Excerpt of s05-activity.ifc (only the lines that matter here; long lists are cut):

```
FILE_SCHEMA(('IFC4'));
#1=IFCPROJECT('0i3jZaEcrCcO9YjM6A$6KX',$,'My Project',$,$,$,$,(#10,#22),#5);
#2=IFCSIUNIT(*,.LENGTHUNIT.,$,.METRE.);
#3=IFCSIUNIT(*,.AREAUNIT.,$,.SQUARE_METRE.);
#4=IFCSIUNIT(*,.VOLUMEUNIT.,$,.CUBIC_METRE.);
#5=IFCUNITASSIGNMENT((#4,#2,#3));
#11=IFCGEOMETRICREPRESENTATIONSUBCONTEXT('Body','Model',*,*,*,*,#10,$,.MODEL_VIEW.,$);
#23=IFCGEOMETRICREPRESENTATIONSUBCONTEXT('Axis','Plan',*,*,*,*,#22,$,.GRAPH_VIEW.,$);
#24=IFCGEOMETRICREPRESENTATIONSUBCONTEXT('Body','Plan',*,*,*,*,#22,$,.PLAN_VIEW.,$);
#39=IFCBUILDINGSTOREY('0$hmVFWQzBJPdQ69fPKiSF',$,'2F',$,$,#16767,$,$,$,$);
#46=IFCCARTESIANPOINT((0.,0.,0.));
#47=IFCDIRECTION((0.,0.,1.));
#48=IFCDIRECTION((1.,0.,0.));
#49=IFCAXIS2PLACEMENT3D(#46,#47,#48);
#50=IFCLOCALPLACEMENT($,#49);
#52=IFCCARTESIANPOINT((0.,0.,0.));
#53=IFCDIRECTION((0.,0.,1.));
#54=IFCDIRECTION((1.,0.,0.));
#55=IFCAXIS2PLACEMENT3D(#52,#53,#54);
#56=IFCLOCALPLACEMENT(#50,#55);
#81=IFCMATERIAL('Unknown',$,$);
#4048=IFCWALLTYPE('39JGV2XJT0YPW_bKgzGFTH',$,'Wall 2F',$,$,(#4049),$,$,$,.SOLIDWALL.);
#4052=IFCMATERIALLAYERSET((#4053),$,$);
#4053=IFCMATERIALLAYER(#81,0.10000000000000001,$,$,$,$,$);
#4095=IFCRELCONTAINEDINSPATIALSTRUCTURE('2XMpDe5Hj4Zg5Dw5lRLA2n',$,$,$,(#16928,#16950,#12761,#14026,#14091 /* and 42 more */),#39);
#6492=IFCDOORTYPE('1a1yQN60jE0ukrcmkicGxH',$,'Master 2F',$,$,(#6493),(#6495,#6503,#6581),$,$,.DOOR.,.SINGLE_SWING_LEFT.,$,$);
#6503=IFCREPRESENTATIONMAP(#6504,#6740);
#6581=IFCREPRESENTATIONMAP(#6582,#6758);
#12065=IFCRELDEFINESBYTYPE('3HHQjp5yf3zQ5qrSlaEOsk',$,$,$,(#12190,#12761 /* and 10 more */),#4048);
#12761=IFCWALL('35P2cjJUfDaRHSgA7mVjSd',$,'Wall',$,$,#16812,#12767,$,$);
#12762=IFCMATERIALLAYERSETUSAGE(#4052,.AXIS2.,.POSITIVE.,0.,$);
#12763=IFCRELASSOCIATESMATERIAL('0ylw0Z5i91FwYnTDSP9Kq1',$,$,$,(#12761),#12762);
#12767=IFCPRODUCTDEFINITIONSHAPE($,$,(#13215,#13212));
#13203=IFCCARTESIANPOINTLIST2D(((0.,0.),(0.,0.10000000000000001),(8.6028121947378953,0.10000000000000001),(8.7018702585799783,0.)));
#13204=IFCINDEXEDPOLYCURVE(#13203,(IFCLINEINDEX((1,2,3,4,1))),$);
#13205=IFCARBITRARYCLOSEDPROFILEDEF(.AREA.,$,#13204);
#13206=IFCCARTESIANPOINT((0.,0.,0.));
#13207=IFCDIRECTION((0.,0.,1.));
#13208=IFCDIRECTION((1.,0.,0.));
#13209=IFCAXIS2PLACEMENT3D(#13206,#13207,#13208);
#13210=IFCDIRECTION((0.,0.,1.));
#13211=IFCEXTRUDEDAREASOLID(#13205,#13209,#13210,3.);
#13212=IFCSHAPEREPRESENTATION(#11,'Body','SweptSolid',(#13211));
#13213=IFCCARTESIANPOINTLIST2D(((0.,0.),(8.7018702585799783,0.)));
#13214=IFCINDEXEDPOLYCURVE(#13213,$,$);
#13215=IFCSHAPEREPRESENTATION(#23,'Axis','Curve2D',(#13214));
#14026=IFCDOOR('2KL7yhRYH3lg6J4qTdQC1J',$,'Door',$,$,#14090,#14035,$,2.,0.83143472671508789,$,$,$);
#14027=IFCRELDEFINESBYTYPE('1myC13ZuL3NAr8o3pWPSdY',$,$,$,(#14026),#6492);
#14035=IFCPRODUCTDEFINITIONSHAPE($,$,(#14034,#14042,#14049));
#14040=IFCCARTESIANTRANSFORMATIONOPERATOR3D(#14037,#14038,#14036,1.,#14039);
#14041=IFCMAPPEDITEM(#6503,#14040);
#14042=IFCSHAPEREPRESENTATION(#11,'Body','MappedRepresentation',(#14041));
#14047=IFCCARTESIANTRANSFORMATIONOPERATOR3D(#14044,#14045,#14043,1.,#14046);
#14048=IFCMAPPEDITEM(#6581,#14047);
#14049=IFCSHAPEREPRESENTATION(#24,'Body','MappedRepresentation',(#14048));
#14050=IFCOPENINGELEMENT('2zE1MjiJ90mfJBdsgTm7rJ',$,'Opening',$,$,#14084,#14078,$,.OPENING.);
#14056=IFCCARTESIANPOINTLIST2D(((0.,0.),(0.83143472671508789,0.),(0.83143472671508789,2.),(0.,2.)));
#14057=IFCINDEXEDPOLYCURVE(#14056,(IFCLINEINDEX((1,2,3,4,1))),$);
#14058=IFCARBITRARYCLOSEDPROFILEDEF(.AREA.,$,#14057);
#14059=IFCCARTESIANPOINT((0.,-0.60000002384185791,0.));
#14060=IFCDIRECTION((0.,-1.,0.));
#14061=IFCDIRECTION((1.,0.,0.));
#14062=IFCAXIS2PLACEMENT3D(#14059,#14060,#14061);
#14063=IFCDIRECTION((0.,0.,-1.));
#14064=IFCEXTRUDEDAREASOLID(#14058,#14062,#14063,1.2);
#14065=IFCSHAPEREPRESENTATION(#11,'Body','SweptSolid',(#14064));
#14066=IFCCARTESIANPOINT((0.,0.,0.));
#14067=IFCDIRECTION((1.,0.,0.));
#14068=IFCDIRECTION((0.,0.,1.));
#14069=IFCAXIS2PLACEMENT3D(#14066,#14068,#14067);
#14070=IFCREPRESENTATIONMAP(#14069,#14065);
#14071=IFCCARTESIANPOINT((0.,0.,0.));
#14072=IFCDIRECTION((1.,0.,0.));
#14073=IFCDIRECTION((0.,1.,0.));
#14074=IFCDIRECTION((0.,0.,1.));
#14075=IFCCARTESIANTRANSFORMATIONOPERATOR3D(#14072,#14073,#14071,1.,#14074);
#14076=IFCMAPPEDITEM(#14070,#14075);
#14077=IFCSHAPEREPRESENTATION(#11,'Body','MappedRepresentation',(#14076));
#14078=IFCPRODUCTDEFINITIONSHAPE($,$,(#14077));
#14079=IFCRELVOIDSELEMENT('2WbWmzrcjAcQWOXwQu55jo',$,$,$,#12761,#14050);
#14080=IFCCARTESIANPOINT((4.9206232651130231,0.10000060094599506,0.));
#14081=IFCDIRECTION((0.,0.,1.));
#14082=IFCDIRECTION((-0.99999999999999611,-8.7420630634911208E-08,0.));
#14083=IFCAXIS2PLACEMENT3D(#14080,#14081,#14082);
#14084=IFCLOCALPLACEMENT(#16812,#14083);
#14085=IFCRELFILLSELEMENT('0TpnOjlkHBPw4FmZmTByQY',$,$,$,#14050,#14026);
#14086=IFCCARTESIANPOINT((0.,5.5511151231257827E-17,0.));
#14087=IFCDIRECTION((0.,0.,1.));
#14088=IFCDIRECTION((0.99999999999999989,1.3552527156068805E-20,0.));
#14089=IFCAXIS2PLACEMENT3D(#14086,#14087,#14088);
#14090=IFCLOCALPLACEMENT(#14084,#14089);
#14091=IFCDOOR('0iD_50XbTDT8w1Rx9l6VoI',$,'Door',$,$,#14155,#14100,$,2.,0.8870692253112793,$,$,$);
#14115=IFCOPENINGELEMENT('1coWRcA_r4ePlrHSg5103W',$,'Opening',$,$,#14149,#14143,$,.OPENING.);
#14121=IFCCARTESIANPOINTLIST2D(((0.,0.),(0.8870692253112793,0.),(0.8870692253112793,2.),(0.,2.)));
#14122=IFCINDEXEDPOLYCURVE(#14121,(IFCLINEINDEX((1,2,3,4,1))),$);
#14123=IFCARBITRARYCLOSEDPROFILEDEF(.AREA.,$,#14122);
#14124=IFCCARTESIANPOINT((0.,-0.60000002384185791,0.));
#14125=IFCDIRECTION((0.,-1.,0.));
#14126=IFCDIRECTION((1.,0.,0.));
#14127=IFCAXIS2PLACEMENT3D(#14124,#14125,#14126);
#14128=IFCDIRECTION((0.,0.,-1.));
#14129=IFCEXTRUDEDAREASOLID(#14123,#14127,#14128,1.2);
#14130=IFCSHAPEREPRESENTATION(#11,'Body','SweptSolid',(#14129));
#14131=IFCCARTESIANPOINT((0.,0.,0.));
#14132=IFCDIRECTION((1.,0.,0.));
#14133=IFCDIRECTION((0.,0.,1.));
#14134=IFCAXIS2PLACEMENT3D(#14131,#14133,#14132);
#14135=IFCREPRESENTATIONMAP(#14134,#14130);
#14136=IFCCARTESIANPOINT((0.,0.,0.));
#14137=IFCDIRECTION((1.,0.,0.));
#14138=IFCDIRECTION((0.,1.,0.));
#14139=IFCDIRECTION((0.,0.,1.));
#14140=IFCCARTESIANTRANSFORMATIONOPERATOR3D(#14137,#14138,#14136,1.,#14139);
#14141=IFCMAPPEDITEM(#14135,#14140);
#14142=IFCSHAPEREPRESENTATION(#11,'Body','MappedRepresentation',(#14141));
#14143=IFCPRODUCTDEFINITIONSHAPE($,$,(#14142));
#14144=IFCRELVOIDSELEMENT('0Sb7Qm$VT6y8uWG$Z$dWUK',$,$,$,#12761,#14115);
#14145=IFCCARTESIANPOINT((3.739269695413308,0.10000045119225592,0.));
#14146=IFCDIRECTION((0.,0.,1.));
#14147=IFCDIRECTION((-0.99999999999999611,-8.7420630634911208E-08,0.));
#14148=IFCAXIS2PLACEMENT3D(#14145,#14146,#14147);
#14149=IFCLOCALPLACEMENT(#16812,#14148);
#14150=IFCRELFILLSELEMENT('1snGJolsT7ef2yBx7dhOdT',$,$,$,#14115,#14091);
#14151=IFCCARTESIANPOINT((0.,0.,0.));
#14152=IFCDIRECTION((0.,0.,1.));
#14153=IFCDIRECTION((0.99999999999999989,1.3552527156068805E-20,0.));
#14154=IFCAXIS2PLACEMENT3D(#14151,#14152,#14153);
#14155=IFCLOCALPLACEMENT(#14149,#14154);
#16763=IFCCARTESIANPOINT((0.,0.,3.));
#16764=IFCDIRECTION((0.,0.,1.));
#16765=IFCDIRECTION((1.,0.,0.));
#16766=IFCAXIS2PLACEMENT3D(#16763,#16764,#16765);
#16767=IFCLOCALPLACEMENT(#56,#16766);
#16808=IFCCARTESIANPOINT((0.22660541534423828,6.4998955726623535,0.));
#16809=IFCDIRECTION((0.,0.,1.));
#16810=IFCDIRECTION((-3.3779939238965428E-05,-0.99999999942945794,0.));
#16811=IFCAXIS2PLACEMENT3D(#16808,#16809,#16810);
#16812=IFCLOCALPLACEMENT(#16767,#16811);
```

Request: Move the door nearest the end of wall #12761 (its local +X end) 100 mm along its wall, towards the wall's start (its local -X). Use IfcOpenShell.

```python
import ifcopenshell
import ifcopenshell.api.geometry
import ifcopenshell.util.placement
import ifcopenshell.util.unit

model = ifcopenshell.open("s05-activity.ifc")
unit_scale = ifcopenshell.util.unit.calculate_unit_scale(model)

door = model.by_guid("2KL7yhRYH3lg6J4qTdQC1J")
opening = door.FillsVoids[0].RelatingOpeningElement
wall = opening.VoidsElements[0].RelatingBuildingElement

wall_matrix = ifcopenshell.util.placement.get_local_placement(wall.ObjectPlacement)
shift = wall_matrix[:3, 0] * -0.1 / unit_scale
before = ifcopenshell.util.placement.get_local_placement(door.ObjectPlacement)[:3, 3].copy()

# The door is placed relative to its opening, so it follows when the opening moves.
matrix = ifcopenshell.util.placement.get_local_placement(opening.ObjectPlacement)
matrix[:3, 3] += shift
ifcopenshell.api.geometry.edit_object_placement(
    model, product=opening, matrix=matrix, is_si=False, should_transform_children=True
)

after = ifcopenshell.util.placement.get_local_placement(door.ObjectPlacement)[:3, 3]
print("door moved by", (after - before).round(3) + 0.0)

model.write("s05-activity-out.ifc")
```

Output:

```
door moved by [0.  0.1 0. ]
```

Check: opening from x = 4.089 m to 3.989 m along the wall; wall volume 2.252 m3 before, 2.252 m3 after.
